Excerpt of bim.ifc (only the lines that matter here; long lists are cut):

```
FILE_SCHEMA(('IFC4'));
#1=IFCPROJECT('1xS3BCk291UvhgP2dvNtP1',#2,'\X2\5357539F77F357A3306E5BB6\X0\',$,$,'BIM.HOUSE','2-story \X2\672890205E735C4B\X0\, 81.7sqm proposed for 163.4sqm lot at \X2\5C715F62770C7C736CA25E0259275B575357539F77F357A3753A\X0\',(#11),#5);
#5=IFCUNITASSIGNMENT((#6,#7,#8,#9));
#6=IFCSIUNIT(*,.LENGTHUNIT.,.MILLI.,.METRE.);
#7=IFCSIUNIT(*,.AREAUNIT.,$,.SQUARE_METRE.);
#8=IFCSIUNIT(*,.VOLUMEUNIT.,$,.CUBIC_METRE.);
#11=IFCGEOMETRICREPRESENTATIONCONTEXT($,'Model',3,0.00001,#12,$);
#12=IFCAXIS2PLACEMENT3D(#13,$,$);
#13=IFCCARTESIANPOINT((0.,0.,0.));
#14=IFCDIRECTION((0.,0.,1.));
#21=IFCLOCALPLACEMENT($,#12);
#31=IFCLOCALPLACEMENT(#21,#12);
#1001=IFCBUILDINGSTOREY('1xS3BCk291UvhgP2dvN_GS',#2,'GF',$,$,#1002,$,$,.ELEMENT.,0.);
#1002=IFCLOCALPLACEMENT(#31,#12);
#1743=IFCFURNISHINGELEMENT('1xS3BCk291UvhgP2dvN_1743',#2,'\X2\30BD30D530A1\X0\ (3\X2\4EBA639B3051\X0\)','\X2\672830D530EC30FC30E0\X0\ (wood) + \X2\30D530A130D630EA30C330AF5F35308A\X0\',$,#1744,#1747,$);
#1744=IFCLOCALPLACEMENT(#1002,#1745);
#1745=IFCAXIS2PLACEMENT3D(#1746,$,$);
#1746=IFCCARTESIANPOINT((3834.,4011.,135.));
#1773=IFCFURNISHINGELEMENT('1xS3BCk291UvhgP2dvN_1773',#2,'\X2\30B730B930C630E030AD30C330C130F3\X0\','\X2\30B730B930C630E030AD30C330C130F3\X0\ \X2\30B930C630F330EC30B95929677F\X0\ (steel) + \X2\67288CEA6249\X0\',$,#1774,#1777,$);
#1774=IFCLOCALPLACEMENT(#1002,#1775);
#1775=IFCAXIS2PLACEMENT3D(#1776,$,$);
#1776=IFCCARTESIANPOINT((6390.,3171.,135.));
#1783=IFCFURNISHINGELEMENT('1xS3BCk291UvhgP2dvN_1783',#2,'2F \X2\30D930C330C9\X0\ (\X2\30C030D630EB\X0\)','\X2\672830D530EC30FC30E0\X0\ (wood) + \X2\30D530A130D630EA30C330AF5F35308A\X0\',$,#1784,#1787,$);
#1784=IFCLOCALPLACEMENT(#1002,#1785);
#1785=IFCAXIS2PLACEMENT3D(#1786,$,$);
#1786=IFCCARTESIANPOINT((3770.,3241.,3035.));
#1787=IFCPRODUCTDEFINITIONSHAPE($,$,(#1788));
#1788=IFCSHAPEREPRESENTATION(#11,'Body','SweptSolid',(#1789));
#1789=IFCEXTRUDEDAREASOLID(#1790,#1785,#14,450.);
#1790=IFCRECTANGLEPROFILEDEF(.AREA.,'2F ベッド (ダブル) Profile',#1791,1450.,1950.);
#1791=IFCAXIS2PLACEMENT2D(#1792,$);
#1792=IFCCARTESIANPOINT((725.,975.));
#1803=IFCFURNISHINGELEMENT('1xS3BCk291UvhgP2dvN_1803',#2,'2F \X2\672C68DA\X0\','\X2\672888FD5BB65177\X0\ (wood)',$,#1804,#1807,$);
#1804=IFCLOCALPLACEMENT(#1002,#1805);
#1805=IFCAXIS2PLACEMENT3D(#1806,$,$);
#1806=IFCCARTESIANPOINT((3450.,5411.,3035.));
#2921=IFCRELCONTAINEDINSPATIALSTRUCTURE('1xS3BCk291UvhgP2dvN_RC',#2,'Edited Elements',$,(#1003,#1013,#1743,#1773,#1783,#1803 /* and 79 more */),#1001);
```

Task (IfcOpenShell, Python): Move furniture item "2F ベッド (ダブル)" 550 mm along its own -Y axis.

```python
import ifcopenshell
import ifcopenshell.api.geometry
import ifcopenshell.util.placement
import ifcopenshell.util.unit

model = ifcopenshell.open("bim.ifc")
unit_scale = ifcopenshell.util.unit.calculate_unit_scale(model)

item = model.by_guid("1xS3BCk291UvhgP2dvN_1783")
matrix = ifcopenshell.util.placement.get_local_placement(item.ObjectPlacement)
matrix[:3, 3] -= matrix[:3, 1] * 0.55 / unit_scale
ifcopenshell.api.geometry.edit_object_placement(model, product=item, matrix=matrix, is_si=False)

print(ifcopenshell.util.placement.get_local_placement(item.ObjectPlacement).round(3) + 0.0)

model.write("bim-out.ifc")
```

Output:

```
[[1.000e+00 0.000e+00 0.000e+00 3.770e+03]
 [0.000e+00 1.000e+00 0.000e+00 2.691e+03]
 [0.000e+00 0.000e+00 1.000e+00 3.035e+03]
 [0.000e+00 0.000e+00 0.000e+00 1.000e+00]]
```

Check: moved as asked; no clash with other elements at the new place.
